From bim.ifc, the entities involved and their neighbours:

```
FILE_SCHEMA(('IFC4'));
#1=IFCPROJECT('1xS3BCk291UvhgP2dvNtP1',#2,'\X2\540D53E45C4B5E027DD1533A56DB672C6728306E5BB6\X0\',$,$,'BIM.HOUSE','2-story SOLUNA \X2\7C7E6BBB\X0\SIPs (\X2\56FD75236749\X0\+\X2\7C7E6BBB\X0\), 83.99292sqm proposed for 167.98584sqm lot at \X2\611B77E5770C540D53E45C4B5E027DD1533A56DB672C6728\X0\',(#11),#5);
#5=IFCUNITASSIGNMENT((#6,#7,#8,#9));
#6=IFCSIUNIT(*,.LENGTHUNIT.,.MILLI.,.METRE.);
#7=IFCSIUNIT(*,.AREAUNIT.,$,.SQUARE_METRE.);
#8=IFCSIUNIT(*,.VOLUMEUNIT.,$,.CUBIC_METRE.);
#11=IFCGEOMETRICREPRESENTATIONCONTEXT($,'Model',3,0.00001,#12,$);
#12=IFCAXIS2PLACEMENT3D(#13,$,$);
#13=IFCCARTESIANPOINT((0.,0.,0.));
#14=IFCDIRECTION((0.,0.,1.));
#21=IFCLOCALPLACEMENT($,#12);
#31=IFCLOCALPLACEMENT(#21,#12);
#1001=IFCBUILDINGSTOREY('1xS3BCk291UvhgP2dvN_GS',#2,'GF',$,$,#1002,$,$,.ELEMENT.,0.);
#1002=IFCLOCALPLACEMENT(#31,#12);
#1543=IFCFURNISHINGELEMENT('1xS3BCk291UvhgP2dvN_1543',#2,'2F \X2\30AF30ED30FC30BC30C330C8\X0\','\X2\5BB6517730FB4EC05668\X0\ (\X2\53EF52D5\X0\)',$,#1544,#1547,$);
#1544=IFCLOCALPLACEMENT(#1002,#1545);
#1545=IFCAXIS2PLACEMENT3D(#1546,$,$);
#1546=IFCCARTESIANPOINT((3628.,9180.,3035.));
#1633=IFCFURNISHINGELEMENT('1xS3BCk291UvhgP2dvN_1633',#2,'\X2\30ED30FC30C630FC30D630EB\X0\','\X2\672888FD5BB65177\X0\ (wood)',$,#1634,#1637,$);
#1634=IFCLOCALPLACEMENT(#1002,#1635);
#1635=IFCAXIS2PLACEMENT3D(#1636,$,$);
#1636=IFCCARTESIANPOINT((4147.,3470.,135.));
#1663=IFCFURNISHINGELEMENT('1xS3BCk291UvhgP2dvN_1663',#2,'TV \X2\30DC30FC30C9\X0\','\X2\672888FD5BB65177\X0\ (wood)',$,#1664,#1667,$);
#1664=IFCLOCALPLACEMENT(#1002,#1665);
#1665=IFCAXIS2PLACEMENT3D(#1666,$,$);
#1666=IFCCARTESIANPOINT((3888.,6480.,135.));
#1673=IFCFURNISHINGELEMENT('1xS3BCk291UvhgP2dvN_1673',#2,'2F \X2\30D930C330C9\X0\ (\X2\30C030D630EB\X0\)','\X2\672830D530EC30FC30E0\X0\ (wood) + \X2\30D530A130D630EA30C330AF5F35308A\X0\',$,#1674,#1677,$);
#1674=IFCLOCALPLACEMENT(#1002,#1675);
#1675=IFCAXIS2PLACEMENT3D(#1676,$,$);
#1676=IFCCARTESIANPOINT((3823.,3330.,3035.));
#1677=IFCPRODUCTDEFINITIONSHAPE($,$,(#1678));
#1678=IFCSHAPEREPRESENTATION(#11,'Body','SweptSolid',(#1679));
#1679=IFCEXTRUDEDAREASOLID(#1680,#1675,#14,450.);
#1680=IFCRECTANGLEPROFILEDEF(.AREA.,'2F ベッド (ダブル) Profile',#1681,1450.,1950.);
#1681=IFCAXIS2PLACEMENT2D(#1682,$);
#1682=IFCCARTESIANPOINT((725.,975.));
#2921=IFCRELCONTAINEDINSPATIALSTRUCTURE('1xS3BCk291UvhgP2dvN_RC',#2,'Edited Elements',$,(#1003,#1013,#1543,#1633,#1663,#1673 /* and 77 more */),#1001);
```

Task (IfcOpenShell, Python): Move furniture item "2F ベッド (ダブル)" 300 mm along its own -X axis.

```python
import ifcopenshell
import ifcopenshell.api.geometry
import ifcopenshell.util.placement
import ifcopenshell.util.unit

model = ifcopenshell.open("bim.ifc")
unit_scale = ifcopenshell.util.unit.calculate_unit_scale(model)

item = model.by_guid("1xS3BCk291UvhgP2dvN_1673")
matrix = ifcopenshell.util.placement.get_local_placement(item.ObjectPlacement)
matrix[:3, 3] -= matrix[:3, 0] * 0.3 / unit_scale
ifcopenshell.api.geometry.edit_object_placement(model, product=item, matrix=matrix, is_si=False)

print(ifcopenshell.util.placement.get_local_placement(item.ObjectPlacement).round(3) + 0.0)

model.write("bim_rev.ifc")
```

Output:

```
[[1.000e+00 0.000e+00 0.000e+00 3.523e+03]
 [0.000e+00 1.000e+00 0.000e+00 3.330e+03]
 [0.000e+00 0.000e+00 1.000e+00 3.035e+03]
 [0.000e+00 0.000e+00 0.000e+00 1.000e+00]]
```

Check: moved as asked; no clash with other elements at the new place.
